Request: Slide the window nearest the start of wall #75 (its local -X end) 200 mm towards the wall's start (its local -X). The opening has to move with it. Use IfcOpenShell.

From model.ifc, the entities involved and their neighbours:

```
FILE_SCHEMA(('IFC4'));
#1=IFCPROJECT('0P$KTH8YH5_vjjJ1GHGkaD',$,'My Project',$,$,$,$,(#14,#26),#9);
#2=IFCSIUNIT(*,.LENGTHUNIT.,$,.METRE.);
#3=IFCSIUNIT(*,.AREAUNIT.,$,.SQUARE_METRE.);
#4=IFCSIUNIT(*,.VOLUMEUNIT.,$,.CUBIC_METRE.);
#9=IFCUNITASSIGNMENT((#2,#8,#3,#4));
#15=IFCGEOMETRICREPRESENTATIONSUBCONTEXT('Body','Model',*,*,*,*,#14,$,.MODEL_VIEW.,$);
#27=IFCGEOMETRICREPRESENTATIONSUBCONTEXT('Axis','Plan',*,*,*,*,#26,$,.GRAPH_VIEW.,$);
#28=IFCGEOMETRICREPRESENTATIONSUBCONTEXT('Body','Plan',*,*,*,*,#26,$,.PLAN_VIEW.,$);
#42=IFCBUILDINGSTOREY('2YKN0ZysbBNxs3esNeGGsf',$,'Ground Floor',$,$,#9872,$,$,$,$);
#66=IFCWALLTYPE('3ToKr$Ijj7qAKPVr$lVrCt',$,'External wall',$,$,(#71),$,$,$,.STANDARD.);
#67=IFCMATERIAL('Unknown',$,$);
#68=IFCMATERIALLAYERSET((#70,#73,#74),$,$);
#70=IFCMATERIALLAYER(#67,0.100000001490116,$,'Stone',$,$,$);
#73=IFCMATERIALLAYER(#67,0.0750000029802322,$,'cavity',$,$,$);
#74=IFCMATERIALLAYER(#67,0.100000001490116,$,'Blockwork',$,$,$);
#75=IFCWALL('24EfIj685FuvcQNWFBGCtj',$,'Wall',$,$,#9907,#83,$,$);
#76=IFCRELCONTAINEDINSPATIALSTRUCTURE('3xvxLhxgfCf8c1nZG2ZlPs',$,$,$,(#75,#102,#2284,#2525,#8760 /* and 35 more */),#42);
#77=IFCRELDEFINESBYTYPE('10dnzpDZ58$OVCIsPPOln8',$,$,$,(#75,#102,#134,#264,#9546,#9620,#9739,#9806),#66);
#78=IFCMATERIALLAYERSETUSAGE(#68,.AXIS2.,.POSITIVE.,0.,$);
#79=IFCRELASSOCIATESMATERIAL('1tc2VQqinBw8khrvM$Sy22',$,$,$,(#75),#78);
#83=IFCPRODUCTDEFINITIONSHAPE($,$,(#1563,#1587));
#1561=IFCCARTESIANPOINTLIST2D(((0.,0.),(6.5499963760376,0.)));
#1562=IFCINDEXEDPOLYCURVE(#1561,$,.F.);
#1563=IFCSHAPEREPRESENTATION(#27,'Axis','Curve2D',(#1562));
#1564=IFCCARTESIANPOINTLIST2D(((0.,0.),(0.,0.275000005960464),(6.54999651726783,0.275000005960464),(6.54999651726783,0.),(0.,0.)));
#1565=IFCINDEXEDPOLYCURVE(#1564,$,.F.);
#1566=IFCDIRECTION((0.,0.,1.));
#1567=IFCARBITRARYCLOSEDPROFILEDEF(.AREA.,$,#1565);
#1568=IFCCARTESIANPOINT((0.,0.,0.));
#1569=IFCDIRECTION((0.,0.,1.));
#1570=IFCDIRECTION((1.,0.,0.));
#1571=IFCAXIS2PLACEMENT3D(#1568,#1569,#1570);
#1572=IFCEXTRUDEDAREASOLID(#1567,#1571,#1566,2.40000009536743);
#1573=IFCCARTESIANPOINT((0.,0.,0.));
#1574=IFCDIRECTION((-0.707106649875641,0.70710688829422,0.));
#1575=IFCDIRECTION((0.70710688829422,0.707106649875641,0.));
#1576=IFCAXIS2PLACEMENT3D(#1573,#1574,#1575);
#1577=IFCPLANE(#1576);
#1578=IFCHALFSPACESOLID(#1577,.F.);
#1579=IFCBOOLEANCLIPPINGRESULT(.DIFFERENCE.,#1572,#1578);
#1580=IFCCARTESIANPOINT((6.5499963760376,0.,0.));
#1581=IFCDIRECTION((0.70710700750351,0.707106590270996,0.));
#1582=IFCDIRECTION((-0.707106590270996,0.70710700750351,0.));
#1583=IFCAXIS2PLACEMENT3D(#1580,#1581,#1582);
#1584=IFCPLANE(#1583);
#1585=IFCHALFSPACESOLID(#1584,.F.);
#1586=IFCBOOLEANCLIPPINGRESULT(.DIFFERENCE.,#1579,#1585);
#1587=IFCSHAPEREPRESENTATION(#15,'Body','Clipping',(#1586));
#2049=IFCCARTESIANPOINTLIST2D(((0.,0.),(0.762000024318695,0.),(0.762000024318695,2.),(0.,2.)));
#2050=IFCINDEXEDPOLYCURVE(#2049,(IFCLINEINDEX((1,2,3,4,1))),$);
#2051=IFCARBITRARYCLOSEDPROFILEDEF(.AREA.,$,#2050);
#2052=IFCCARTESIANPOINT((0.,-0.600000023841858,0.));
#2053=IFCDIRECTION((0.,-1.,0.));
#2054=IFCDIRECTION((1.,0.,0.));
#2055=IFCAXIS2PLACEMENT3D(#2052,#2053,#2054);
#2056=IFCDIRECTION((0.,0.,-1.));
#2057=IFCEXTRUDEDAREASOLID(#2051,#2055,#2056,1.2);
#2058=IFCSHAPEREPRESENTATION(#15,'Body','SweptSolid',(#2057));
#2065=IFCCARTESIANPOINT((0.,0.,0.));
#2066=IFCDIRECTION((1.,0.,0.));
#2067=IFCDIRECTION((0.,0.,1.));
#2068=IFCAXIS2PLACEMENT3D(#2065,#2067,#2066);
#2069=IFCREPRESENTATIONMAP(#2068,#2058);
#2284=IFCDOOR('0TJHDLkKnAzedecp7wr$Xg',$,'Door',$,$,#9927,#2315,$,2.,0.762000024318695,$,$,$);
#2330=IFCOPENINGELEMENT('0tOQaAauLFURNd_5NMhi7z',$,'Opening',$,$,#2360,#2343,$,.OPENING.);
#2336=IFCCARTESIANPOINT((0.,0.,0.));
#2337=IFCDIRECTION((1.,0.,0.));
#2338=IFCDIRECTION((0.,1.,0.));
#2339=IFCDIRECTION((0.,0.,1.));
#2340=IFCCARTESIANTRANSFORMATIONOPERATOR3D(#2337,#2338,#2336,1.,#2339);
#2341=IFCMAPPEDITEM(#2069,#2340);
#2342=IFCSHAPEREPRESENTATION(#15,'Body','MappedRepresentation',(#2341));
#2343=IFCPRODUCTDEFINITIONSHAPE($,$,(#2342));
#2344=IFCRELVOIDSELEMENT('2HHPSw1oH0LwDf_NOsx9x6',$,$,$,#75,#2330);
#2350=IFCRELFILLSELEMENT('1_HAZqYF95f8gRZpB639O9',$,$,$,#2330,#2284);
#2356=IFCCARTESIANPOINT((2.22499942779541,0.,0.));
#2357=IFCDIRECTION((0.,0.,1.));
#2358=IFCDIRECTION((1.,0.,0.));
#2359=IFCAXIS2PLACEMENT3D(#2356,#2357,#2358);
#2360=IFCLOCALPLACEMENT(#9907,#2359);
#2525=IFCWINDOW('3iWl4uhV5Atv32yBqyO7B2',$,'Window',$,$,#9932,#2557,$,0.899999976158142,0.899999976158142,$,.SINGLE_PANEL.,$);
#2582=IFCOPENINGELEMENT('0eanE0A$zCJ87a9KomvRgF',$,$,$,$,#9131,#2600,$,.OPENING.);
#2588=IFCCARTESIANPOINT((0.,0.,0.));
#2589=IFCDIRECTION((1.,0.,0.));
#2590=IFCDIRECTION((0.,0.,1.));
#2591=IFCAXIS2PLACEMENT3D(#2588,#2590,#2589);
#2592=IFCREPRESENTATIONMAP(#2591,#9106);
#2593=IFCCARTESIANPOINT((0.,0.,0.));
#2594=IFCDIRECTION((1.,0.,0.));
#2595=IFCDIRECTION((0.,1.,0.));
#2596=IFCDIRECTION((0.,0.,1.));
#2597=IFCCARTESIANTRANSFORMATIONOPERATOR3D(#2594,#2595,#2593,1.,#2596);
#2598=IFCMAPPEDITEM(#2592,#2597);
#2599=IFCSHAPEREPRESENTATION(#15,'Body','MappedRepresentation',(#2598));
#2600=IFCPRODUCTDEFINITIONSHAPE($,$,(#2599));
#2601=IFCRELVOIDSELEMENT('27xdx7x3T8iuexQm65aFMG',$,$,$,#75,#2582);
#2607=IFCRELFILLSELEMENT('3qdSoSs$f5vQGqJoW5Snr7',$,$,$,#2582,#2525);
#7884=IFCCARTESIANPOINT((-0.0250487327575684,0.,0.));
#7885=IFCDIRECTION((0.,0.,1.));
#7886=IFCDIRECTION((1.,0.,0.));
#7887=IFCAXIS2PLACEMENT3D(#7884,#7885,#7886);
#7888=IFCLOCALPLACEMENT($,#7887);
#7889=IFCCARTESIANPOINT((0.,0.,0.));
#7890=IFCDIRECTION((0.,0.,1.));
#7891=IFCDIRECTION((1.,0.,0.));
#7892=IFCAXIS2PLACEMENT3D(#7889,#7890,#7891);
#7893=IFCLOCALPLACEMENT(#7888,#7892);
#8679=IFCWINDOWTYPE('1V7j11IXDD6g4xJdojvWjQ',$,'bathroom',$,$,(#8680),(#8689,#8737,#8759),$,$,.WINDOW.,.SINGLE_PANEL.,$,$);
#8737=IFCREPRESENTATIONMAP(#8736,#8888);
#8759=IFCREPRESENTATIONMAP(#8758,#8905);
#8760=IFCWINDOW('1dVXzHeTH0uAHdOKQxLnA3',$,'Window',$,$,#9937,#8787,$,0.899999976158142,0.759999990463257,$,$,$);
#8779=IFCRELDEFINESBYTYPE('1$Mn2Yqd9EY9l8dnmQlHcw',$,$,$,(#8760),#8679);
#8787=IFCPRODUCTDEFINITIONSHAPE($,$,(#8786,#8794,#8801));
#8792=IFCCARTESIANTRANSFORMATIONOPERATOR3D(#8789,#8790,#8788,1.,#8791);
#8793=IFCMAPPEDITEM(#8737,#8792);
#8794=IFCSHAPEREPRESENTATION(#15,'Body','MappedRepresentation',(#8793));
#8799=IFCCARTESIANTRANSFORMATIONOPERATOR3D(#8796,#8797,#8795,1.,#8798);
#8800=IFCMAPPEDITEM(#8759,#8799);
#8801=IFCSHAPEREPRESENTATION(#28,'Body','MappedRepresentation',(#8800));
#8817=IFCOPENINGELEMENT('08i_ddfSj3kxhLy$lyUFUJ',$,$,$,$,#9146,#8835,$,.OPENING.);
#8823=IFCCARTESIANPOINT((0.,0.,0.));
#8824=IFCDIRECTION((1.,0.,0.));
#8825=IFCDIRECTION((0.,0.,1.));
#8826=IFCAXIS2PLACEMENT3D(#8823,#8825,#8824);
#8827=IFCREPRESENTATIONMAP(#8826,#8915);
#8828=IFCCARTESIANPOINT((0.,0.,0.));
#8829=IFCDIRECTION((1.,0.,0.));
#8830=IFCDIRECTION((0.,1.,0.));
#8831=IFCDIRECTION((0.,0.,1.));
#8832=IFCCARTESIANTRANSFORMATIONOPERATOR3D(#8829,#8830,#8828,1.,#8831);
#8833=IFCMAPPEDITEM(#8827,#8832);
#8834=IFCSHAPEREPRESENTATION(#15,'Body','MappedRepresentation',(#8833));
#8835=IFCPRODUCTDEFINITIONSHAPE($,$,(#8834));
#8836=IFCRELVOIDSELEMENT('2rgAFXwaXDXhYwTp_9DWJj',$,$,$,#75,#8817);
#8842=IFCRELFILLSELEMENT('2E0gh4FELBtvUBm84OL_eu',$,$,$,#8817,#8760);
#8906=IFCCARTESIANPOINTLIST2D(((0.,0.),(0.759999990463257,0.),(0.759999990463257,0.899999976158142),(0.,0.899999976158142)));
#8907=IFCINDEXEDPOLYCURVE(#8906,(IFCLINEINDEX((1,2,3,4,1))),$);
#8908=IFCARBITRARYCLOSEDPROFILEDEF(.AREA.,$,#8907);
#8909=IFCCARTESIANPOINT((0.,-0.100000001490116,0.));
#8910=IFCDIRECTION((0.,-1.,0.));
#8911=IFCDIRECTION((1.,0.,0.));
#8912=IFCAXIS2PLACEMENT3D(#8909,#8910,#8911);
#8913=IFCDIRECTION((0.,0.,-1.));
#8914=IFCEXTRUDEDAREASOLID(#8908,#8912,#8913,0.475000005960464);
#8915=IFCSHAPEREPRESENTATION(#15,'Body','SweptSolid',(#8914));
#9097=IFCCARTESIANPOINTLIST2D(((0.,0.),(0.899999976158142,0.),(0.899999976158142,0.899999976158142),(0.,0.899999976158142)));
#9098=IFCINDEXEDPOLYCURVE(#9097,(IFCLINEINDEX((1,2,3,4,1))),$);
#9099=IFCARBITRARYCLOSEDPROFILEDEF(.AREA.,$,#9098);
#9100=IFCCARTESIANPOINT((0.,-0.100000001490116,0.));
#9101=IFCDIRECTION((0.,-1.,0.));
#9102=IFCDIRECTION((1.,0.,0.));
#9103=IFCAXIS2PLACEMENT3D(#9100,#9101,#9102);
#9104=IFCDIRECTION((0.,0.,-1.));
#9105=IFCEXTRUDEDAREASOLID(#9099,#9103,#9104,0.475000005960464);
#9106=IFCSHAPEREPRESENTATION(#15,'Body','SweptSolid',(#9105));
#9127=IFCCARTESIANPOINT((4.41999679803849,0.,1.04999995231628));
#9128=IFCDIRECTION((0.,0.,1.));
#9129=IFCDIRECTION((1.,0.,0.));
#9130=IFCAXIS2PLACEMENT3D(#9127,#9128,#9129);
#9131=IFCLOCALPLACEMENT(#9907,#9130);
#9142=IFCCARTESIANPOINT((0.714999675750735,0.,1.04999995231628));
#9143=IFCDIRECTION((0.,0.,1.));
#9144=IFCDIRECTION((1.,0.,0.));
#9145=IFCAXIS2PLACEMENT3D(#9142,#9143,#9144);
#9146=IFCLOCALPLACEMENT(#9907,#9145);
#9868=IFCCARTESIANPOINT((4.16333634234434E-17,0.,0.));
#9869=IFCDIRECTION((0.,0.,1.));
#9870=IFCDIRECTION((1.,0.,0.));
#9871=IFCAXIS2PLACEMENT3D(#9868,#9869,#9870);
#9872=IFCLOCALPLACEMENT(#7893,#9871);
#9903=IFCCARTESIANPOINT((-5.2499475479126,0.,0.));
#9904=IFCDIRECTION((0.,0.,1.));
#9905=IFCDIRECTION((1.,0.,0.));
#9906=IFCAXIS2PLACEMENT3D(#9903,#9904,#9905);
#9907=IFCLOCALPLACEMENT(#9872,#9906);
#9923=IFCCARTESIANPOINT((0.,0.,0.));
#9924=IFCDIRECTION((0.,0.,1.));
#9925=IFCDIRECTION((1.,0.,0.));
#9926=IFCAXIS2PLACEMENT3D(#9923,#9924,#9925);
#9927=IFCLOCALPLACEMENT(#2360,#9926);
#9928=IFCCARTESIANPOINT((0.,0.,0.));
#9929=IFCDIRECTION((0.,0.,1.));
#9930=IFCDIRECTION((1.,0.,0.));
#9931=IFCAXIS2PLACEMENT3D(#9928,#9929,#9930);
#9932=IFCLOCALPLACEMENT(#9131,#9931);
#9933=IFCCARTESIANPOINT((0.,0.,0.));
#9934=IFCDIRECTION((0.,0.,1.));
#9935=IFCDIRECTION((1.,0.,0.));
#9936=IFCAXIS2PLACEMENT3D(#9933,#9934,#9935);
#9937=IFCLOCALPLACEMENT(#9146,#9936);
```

```python
import ifcopenshell
import ifcopenshell.api.geometry
import ifcopenshell.util.placement

model = ifcopenshell.open("model.ifc")

window = model.by_id(8760)
opening = window.FillsVoids[0].RelatingOpeningElement
wall = opening.VoidsElements[0].RelatingBuildingElement

wall_matrix = ifcopenshell.util.placement.get_local_placement(wall.ObjectPlacement)
shift = wall_matrix[:3, 0] * -0.2
before = ifcopenshell.util.placement.get_local_placement(window.ObjectPlacement)[:3, 3].copy()

# The window is placed relative to its opening, so it follows when the opening moves.
matrix = ifcopenshell.util.placement.get_local_placement(opening.ObjectPlacement)
matrix[:3, 3] += shift
ifcopenshell.api.geometry.edit_object_placement(
    model, product=opening, matrix=matrix, is_si=False, should_transform_children=True
)

after = ifcopenshell.util.placement.get_local_placement(window.ObjectPlacement)[:3, 3]
print("window moved by", (after - before).round(3) + 0.0)

model.write("model_v2.ifc")
```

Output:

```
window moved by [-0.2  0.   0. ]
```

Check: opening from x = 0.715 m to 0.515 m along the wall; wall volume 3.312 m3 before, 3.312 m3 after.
